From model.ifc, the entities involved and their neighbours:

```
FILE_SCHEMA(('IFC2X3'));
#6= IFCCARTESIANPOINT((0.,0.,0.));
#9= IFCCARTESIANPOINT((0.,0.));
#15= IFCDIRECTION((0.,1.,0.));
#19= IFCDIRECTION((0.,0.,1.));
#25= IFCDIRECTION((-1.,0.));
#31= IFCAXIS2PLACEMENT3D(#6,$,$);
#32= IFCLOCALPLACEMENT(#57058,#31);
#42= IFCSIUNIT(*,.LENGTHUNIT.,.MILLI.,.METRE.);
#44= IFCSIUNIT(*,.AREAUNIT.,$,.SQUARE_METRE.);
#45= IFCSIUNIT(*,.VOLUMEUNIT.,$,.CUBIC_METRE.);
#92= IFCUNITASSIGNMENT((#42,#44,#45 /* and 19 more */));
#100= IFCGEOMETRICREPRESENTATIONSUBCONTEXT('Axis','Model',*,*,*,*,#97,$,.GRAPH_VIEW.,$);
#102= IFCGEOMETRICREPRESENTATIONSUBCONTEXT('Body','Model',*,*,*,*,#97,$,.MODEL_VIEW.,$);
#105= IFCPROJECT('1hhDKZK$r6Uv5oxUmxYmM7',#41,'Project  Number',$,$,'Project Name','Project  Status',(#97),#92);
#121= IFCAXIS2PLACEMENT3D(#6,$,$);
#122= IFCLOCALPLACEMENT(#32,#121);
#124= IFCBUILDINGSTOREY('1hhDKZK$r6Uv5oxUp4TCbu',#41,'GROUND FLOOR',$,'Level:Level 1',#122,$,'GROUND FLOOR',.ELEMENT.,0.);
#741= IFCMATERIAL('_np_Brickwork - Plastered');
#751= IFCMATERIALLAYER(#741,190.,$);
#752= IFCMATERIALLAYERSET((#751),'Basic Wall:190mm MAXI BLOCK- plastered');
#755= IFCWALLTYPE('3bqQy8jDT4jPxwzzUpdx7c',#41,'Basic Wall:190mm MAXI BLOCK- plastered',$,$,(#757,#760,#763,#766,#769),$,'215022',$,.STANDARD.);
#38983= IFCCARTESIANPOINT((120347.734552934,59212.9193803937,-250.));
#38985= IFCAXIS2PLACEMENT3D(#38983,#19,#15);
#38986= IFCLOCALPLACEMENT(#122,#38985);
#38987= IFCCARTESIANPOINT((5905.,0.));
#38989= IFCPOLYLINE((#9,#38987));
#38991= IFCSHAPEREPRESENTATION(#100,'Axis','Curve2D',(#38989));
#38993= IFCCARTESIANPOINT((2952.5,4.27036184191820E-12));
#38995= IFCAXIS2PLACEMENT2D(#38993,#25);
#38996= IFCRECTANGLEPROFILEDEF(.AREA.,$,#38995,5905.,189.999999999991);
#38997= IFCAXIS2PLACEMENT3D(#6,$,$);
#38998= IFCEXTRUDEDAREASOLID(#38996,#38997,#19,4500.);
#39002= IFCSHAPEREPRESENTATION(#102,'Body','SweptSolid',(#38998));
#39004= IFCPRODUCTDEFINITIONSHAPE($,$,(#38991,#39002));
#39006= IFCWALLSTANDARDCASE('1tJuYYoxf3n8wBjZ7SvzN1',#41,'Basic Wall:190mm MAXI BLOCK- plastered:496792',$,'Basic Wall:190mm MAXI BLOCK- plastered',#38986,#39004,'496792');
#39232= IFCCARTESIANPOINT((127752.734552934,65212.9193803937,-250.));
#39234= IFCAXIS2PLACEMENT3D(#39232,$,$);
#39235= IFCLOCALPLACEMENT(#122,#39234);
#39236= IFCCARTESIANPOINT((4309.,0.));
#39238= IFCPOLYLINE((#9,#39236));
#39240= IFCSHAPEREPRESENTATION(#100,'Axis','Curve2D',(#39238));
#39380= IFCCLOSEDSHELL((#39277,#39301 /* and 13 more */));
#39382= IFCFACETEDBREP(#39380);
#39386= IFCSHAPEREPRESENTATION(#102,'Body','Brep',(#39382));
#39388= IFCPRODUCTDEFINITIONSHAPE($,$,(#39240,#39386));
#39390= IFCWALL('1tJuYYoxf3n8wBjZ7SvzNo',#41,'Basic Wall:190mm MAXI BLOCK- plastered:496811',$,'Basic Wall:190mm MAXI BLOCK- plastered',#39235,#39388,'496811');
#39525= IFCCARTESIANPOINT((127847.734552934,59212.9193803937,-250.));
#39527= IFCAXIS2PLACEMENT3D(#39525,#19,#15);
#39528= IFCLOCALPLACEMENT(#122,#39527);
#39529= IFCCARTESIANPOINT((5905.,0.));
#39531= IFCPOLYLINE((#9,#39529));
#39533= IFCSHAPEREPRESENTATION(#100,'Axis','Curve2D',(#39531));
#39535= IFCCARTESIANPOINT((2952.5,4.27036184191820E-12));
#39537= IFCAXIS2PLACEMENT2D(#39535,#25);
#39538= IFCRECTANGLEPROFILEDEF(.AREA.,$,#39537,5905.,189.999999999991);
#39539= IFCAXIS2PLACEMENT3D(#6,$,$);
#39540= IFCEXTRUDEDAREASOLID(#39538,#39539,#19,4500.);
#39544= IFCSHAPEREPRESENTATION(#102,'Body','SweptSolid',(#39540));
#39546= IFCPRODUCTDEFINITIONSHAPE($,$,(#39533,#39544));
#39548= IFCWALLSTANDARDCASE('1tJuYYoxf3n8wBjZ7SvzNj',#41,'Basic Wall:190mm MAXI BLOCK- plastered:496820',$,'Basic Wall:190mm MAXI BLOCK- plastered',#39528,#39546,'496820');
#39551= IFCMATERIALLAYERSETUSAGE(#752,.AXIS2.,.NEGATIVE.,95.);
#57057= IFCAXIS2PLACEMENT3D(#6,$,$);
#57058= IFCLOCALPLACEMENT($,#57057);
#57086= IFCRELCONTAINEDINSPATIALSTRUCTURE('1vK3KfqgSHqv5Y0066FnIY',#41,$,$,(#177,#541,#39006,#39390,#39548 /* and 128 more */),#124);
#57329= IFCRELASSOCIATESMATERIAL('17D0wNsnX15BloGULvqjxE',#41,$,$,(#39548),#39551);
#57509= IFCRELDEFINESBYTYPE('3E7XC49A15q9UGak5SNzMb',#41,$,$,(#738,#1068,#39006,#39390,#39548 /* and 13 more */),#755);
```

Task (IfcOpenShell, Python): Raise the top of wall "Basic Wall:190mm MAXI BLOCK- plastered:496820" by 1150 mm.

```python
import ifcopenshell
import ifcopenshell.geom
import ifcopenshell.util.representation
import ifcopenshell.util.shape

model = ifcopenshell.open("model.ifc")
settings = ifcopenshell.geom.settings()


def volume(element):
    """Net volume in cubic metres, openings subtracted."""
    shape = ifcopenshell.geom.create_shape(settings, element)
    return ifcopenshell.util.shape.get_volume(shape.geometry)


wall = model.by_guid("1tJuYYoxf3n8wBjZ7SvzNj")
before = volume(wall)

body = ifcopenshell.util.representation.get_representation(wall, "Model", "Body")
solid = body.Items[0]
old_height = solid.Depth
solid.Depth += 1150.0
after = volume(wall)

print(f"height {old_height:g} -> {solid.Depth:g}, volume {before:.3f} -> {after:.3f} m3")

model.write("model-out.ifc")
```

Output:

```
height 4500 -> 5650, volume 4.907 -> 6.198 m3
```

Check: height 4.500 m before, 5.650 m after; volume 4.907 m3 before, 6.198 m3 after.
